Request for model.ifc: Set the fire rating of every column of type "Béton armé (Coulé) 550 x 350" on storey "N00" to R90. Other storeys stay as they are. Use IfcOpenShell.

First a look at what the model holds.

```python
import ifcopenshell
import ifcopenshell.util.element

model = ifcopenshell.open("model.ifc")
print(model.schema)
storey = next(s for s in model.by_type("IfcBuildingStorey") if s.Name == "N00")
columns = [e for e in ifcopenshell.util.element.get_decomposition(storey) if e.is_a("IfcColumn")]
seen = {}
for e in columns:
    element_type = ifcopenshell.util.element.get_type(e)
    key = (element_type.Name if element_type != e and element_type else None, ifcopenshell.util.element.get_pset(e, "Pset_ColumnCommon", "FireRating"))
    seen[key] = seen.get(key, 0) + 1
for (name, value), count in sorted(seen.items(), key=str):
    print(count, "x", name, "|", value)
```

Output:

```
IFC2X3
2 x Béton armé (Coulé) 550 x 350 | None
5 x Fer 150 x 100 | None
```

```python
import ifcopenshell
import ifcopenshell.api.pset
import ifcopenshell.util.element

model = ifcopenshell.open("model.ifc")

storey = next(s for s in model.by_type("IfcBuildingStorey") if s.Name == "N00")
columns = [e for e in ifcopenshell.util.element.get_decomposition(storey) if e.is_a("IfcColumn")]

count = 0
for e in columns:
    element_type = ifcopenshell.util.element.get_type(e)
    if element_type in (None, e) or element_type.Name != "Béton armé (Coulé) 550 x 350":
        continue
    # add_pset returns the element's existing set when there is one.
    pset = ifcopenshell.api.pset.add_pset(model, product=e, name="Pset_ColumnCommon")
    ifcopenshell.api.pset.edit_pset(model, pset=pset, properties={"FireRating": "R90"})
    count += 1

print(count, "columns updated")

model.write("model_rev.ifc")
```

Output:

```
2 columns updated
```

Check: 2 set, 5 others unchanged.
